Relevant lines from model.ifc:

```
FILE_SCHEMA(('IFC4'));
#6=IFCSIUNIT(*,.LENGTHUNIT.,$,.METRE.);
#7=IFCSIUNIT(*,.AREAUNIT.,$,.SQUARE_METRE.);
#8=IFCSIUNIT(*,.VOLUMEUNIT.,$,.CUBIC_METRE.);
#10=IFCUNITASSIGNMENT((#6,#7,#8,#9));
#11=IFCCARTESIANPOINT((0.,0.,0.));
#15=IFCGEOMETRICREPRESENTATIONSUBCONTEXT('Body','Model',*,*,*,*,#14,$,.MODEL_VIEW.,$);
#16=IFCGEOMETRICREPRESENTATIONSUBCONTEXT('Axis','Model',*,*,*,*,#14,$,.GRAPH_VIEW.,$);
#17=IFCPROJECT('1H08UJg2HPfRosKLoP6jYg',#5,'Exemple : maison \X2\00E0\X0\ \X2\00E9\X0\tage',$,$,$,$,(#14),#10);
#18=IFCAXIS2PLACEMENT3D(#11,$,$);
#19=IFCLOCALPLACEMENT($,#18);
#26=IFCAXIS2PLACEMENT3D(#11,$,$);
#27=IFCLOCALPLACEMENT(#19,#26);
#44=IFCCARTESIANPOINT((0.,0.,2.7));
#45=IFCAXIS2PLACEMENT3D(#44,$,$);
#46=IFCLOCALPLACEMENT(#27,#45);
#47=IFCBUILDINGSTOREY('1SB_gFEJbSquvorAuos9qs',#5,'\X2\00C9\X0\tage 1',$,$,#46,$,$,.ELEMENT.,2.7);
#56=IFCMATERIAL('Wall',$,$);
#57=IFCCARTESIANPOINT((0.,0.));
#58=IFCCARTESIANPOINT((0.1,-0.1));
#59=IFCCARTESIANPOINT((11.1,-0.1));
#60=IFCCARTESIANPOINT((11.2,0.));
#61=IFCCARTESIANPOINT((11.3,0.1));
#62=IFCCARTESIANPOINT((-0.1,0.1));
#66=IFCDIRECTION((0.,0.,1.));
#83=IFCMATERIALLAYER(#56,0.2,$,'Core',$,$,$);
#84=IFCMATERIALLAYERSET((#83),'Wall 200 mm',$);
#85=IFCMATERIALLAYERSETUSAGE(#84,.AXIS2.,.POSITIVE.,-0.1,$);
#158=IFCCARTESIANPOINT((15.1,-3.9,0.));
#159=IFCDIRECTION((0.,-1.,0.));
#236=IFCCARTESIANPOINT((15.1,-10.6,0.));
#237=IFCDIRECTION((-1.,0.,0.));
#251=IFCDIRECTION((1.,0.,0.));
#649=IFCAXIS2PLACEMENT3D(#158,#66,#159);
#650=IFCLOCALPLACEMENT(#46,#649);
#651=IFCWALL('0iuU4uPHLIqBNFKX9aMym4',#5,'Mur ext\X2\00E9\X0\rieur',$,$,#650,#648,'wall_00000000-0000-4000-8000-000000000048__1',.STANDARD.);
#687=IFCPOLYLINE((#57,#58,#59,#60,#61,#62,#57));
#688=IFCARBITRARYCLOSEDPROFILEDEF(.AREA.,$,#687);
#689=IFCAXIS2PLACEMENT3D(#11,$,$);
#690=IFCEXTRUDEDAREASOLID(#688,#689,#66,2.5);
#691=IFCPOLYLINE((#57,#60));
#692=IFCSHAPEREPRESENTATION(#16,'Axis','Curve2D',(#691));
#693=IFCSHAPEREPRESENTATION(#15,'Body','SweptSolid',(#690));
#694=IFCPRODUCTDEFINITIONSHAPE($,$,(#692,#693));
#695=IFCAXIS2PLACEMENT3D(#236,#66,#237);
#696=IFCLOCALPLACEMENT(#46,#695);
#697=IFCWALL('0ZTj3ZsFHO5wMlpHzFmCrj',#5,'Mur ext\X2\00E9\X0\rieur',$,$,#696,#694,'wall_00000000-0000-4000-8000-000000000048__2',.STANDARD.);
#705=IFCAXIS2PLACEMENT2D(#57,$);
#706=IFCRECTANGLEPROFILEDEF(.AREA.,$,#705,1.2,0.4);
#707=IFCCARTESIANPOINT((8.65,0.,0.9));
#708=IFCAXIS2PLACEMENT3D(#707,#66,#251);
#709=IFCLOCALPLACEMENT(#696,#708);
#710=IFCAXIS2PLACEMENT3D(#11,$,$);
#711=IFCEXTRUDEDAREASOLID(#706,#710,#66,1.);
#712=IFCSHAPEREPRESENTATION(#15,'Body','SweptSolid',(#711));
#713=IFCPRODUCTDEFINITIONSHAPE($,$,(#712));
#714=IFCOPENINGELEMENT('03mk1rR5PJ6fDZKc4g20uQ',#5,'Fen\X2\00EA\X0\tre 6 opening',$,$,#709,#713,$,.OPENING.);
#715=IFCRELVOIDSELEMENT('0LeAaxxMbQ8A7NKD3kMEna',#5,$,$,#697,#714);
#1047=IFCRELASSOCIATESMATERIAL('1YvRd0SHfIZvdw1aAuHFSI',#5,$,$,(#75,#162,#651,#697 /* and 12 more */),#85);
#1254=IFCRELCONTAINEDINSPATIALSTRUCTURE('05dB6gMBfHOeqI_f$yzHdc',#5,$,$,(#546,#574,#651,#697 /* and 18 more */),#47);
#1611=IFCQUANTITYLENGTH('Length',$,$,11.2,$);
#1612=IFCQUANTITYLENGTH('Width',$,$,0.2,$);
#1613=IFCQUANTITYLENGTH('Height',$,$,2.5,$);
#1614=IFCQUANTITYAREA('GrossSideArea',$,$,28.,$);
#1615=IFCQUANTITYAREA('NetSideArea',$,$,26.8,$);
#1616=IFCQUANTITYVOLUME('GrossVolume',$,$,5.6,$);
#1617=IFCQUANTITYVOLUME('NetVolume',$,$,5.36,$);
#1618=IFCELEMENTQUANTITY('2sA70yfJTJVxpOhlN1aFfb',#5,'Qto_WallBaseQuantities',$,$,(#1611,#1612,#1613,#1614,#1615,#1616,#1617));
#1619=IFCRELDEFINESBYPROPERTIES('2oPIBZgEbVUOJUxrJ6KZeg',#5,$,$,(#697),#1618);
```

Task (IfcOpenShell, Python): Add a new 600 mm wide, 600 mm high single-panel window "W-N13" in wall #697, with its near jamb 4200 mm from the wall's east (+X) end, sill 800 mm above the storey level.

```python
import numpy as np
import ifcopenshell
import ifcopenshell.api.feature
import ifcopenshell.api.geometry
import ifcopenshell.api.pset
import ifcopenshell.api.root
import ifcopenshell.api.spatial
import ifcopenshell.geom
import ifcopenshell.util.element
import ifcopenshell.util.placement
import ifcopenshell.util.representation
import ifcopenshell.util.shape
import ifcopenshell.util.unit

model = ifcopenshell.open("model.ifc")
unit_scale = ifcopenshell.util.unit.calculate_unit_scale(model)
area_scale = ifcopenshell.util.unit.calculate_unit_scale(model, "AREAUNIT")
volume_scale = ifcopenshell.util.unit.calculate_unit_scale(model, "VOLUMEUNIT")
settings = ifcopenshell.geom.settings()


def volume(element):
    """Net volume in cubic metres, openings subtracted."""
    shape = ifcopenshell.geom.create_shape(settings, element)
    return ifcopenshell.util.shape.get_volume(shape.geometry)


wall = model.by_guid("0ZTj3ZsFHO5wMlpHzFmCrj")
storey = ifcopenshell.util.element.get_container(wall, ifc_class="IfcBuildingStorey")
context = ifcopenshell.util.representation.get_context(model, "Model", "Body", "MODEL_VIEW")
before = volume(wall)

width, height, from_end, sill = 0.6, 0.6, 4.2, 0.8  # metres

# The wall runs along its own X axis, and the end named is its -X end.
wall_shape = ifcopenshell.geom.create_shape(settings, wall)
x, y, z = ifcopenshell.util.shape.get_vertices(wall_shape.geometry).T
start = x.min() + from_end
face, thickness = float(y.min()), float(y.max() - y.min())
wall_matrix = ifcopenshell.util.placement.get_local_placement(wall.ObjectPlacement)
level = ifcopenshell.util.placement.get_local_placement(storey.ObjectPlacement)[2, 3]


def in_wall(x, y):
    """Placement at x, y metres in the wall's axes, at sill height."""
    matrix = wall_matrix.copy()
    matrix[:, 3] = wall_matrix @ np.array([x / unit_scale, y / unit_scale, 0.0, 1.0])
    matrix[2, 3] = level + sill / unit_scale
    return matrix


# Opening: a box that overshoots both wall faces by 50 mm.
opening = ifcopenshell.api.root.create_entity(model, ifc_class="IfcOpeningElement", predefined_type="OPENING")
box = ifcopenshell.api.geometry.add_wall_representation(
    model, context=context, length=width, height=height, thickness=thickness + 0.1
)
ifcopenshell.api.geometry.assign_representation(model, product=opening, representation=box)
ifcopenshell.api.geometry.edit_object_placement(model, product=opening, matrix=in_wall(start, face - 0.05), is_si=False)
ifcopenshell.api.feature.add_feature(model, feature=opening, element=wall)

window = ifcopenshell.api.root.create_entity(model, ifc_class="IfcWindow", name="W-N13", predefined_type="WINDOW")
window.OverallWidth, window.OverallHeight = width / unit_scale, height / unit_scale
window.PartitioningType = "SINGLE_PANEL"
body = ifcopenshell.api.geometry.add_window_representation(
    model,
    context=context,
    overall_width=window.OverallWidth,
    overall_height=window.OverallHeight,
    partition_type="SINGLE_PANEL",
)
ifcopenshell.api.geometry.assign_representation(model, product=window, representation=body)
ifcopenshell.api.spatial.assign_container(model, products=[window], relating_structure=storey)
ifcopenshell.api.feature.add_filling(model, opening=opening, element=window)

# Centre the window in the wall's thickness.
ifcopenshell.api.geometry.edit_object_placement(model, product=window, matrix=in_wall(start, face), is_si=False)
window_shape = ifcopenshell.geom.create_shape(settings, window)
depth = ifcopenshell.util.shape.get_vertices(window_shape.geometry)[:, 1]
offset = face + thickness / 2 - (depth.min() + depth.max()) / 2
ifcopenshell.api.geometry.edit_object_placement(model, product=window, matrix=in_wall(start, offset), is_si=False)

after = volume(wall)

# Update the wall's stored quantities.
qto = model.by_id(ifcopenshell.util.element.get_pset(wall, "Qto_WallBaseQuantities", should_inherit=False)["id"])
ifcopenshell.api.pset.edit_qto(model, qto=qto, properties={
    "NetSideArea": after / thickness / area_scale,
    "NetVolume": after / volume_scale,
})

print(f"wall volume {before:.3f} -> {after:.3f} m3")

model.write("model_updated.ifc")
```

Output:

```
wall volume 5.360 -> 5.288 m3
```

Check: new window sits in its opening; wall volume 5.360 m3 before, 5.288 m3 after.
